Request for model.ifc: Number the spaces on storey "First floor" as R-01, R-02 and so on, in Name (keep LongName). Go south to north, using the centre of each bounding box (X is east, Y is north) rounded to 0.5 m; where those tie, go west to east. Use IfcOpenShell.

First a look at what the model holds.

```python
import ifcopenshell
import ifcopenshell.util.element
import ifcopenshell.util.placement

model = ifcopenshell.open("model.ifc")
print(model.schema)
storey = next(s for s in model.by_type("IfcBuildingStorey") if s.Name == "First floor")
spaces = [e for e in ifcopenshell.util.element.get_decomposition(storey) if e.is_a("IfcSpace")]
for e in sorted(spaces, key=lambda e: e.id()):
    origin = ifcopenshell.util.placement.get_local_placement(e.ObjectPlacement)[:3, 3]
    print(e.id(), e.Name, e.LongName, origin.round(2) + 0.0, sep=" | ")
```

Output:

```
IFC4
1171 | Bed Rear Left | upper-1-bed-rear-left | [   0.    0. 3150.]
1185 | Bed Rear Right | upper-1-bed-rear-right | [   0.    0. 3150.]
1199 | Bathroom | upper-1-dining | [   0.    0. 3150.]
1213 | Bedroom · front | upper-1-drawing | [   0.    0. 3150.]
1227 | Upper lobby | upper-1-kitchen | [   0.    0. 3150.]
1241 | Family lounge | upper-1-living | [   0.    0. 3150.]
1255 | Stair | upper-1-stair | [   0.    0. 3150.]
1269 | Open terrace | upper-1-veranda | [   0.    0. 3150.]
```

```python
import ifcopenshell
import ifcopenshell.geom
import ifcopenshell.util.element
import ifcopenshell.util.shape

model = ifcopenshell.open("model.ifc")
settings = ifcopenshell.geom.settings()
settings.set("use-world-coords", True)


def centre(element):
    shape = ifcopenshell.geom.create_shape(settings, element)
    return ifcopenshell.util.shape.get_bbox_centroid(shape.geometry)


storey = next(s for s in model.by_type("IfcBuildingStorey") if s.Name == "First floor")
spaces = [e for e in ifcopenshell.util.element.get_decomposition(storey) if e.is_a("IfcSpace")]

# Insertion points can sit at a corner or the storey origin, so sort by the geometry (in metres).
centres = {e: centre(e) for e in spaces}
spaces.sort(key=lambda e: (round(centres[e][1] / 0.5), centres[e][0]))

for i, e in enumerate(spaces, start=1):
    number = f"R-{i:02d}"
    e.Name = number
    print(e.id(), number)

model.write("model_updated.ifc")
```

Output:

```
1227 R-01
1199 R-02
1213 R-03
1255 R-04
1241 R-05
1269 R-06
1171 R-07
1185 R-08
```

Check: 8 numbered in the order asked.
